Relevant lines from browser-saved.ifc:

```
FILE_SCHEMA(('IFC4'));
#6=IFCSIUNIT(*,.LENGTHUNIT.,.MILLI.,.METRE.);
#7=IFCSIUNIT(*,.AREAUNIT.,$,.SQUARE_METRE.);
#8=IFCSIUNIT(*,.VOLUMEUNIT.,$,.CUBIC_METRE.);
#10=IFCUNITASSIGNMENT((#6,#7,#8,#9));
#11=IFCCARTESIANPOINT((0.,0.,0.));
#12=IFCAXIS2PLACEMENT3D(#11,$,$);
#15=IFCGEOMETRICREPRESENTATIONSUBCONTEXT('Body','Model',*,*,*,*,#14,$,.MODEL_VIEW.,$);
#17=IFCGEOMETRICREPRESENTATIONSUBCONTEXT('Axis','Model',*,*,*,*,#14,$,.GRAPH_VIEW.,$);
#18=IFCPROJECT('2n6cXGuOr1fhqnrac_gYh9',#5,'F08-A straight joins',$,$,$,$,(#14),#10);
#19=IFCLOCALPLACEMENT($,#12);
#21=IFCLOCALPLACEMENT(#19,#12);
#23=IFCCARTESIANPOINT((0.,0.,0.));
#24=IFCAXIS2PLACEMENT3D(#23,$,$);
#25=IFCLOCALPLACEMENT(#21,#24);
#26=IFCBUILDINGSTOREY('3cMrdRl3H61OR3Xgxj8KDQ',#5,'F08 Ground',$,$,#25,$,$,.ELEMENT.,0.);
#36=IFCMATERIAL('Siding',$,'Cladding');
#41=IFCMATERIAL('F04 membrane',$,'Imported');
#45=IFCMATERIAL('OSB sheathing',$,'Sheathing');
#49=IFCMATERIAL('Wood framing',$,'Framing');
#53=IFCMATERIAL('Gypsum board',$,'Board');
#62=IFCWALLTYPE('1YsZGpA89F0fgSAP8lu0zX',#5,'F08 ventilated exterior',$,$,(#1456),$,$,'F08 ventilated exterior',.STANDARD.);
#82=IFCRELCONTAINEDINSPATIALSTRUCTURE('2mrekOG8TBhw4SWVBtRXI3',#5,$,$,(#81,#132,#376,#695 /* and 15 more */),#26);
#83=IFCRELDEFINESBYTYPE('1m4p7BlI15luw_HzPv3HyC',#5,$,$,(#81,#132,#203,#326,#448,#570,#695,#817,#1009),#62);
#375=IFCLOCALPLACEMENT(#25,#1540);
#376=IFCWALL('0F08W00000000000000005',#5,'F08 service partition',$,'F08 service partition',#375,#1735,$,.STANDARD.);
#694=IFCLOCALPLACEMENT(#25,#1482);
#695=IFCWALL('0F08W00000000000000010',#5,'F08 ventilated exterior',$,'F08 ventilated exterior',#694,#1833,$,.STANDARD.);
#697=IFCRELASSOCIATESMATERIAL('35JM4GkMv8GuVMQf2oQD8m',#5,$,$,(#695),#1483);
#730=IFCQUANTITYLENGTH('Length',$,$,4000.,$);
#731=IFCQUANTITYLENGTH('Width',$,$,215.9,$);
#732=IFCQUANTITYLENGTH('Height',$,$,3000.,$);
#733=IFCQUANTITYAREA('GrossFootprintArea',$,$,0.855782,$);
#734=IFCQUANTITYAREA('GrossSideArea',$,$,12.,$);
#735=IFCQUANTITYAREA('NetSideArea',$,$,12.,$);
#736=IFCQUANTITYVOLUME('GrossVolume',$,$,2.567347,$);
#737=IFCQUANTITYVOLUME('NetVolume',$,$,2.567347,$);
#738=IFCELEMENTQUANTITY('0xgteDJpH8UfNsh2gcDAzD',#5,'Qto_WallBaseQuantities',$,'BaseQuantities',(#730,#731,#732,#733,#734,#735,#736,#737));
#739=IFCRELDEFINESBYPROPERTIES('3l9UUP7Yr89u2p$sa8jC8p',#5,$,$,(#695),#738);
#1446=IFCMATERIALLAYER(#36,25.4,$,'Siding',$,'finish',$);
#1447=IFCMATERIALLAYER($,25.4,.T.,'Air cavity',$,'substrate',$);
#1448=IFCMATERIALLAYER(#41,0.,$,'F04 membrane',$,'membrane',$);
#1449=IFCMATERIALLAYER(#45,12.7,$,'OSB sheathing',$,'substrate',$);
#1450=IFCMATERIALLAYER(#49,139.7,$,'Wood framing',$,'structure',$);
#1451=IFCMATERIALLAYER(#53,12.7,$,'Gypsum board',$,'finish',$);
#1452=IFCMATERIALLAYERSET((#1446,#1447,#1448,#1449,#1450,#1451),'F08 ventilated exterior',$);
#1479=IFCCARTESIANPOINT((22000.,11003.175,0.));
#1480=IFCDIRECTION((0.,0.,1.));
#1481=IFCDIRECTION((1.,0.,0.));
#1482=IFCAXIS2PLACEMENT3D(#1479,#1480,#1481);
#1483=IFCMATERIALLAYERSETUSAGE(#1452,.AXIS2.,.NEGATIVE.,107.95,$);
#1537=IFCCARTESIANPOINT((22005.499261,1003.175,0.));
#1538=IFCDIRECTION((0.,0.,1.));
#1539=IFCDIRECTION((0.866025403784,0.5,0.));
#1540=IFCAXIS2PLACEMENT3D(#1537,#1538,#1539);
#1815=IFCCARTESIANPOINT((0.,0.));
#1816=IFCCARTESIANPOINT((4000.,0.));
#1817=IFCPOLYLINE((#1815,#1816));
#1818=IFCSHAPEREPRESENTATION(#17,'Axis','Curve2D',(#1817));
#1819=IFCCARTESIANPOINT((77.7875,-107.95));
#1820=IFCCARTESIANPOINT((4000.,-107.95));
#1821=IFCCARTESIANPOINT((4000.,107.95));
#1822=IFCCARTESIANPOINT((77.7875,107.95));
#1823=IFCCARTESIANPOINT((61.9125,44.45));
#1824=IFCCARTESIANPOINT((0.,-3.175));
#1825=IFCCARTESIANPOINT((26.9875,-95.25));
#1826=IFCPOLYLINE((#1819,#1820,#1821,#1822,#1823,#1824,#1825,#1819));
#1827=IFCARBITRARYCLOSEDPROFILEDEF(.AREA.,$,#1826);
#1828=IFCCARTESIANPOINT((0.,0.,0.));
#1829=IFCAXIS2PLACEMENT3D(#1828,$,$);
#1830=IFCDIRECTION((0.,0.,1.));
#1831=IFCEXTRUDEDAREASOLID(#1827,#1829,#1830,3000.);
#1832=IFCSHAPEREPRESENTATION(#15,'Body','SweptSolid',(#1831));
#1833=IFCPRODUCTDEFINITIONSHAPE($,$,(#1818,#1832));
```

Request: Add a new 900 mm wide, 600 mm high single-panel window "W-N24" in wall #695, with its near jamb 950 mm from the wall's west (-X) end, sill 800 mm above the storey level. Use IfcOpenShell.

```python
import numpy as np
import ifcopenshell
import ifcopenshell.api.feature
import ifcopenshell.api.geometry
import ifcopenshell.api.pset
import ifcopenshell.api.root
import ifcopenshell.api.spatial
import ifcopenshell.geom
import ifcopenshell.util.element
import ifcopenshell.util.placement
import ifcopenshell.util.representation
import ifcopenshell.util.shape
import ifcopenshell.util.unit

model = ifcopenshell.open("browser-saved.ifc")
unit_scale = ifcopenshell.util.unit.calculate_unit_scale(model)
area_scale = ifcopenshell.util.unit.calculate_unit_scale(model, "AREAUNIT")
volume_scale = ifcopenshell.util.unit.calculate_unit_scale(model, "VOLUMEUNIT")
settings = ifcopenshell.geom.settings()


def volume(element):
    """Net volume in cubic metres, openings subtracted."""
    shape = ifcopenshell.geom.create_shape(settings, element)
    return ifcopenshell.util.shape.get_volume(shape.geometry)


wall = model.by_id(695)
storey = ifcopenshell.util.element.get_container(wall, ifc_class="IfcBuildingStorey")
context = ifcopenshell.util.representation.get_context(model, "Model", "Body", "MODEL_VIEW")
before = volume(wall)

width, height, from_end, sill = 0.9, 0.6, 0.95, 0.8  # metres

# The wall runs along its own X axis, and the end named is its -X end.
wall_shape = ifcopenshell.geom.create_shape(settings, wall)
x, y, z = ifcopenshell.util.shape.get_vertices(wall_shape.geometry).T
start = x.min() + from_end
face, thickness = float(y.min()), float(y.max() - y.min())
wall_matrix = ifcopenshell.util.placement.get_local_placement(wall.ObjectPlacement)
level = ifcopenshell.util.placement.get_local_placement(storey.ObjectPlacement)[2, 3]


def in_wall(x, y):
    """Placement at x, y metres in the wall's axes, at sill height."""
    matrix = wall_matrix.copy()
    matrix[:, 3] = wall_matrix @ np.array([x / unit_scale, y / unit_scale, 0.0, 1.0])
    matrix[2, 3] = level + sill / unit_scale
    return matrix


# Opening: a box that overshoots both wall faces by 50 mm.
opening = ifcopenshell.api.root.create_entity(model, ifc_class="IfcOpeningElement", predefined_type="OPENING")
box = ifcopenshell.api.geometry.add_wall_representation(
    model, context=context, length=width, height=height, thickness=thickness + 0.1
)
ifcopenshell.api.geometry.assign_representation(model, product=opening, representation=box)
ifcopenshell.api.geometry.edit_object_placement(model, product=opening, matrix=in_wall(start, face - 0.05), is_si=False)
ifcopenshell.api.feature.add_feature(model, feature=opening, element=wall)

window = ifcopenshell.api.root.create_entity(model, ifc_class="IfcWindow", name="W-N24", predefined_type="WINDOW")
window.OverallWidth, window.OverallHeight = width / unit_scale, height / unit_scale
window.PartitioningType = "SINGLE_PANEL"
body = ifcopenshell.api.geometry.add_window_representation(
    model,
    context=context,
    overall_width=window.OverallWidth,
    overall_height=window.OverallHeight,
    partition_type="SINGLE_PANEL",
)
ifcopenshell.api.geometry.assign_representation(model, product=window, representation=body)
ifcopenshell.api.spatial.assign_container(model, products=[window], relating_structure=storey)
ifcopenshell.api.feature.add_filling(model, opening=opening, element=window)

# Centre the window in the wall's thickness.
ifcopenshell.api.geometry.edit_object_placement(model, product=window, matrix=in_wall(start, face), is_si=False)
window_shape = ifcopenshell.geom.create_shape(settings, window)
depth = ifcopenshell.util.shape.get_vertices(window_shape.geometry)[:, 1]
offset = face + thickness / 2 - (depth.min() + depth.max()) / 2
ifcopenshell.api.geometry.edit_object_placement(model, product=window, matrix=in_wall(start, offset), is_si=False)

after = volume(wall)

# Update the wall's stored quantities.
qto = model.by_id(ifcopenshell.util.element.get_pset(wall, "Qto_WallBaseQuantities", should_inherit=False)["id"])
ifcopenshell.api.pset.edit_qto(model, qto=qto, properties={
    "NetSideArea": after / thickness / area_scale,
    "NetVolume": after / volume_scale,
})

print(f"wall volume {before:.3f} -> {after:.3f} m3")

model.write("browser-saved_rev.ifc")
```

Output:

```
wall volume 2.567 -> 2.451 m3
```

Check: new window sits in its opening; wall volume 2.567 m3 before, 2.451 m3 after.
